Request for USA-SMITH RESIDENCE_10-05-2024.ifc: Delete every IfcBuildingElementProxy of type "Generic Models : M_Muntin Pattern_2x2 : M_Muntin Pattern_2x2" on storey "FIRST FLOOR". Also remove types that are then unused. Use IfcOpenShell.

First a look at what the model holds.

```python
import ifcopenshell
import ifcopenshell.util.element

model = ifcopenshell.open("USA-SMITH RESIDENCE_10-05-2024.ifc")
print(model.schema)
storey = next(s for s in model.by_type("IfcBuildingStorey") if s.Name == "FIRST FLOOR")
proxies = [e for e in ifcopenshell.util.element.get_decomposition(storey) if e.is_a("IfcBuildingElementProxy")]
seen = {}
for e in proxies:
    element_type = ifcopenshell.util.element.get_type(e)
    name = element_type.Name if element_type not in (None, e) else None
    seen[name] = seen.get(name, 0) + 1
for name, count in sorted(seen.items(), key=str):
    print(count, "x", name)
```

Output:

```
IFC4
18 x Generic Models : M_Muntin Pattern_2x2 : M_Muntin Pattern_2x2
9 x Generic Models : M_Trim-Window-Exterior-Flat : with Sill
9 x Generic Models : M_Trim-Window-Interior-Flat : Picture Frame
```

```python
import ifcopenshell
import ifcopenshell.api.root
import ifcopenshell.util.element

model = ifcopenshell.open("USA-SMITH RESIDENCE_10-05-2024.ifc")

storey = next(s for s in model.by_type("IfcBuildingStorey") if s.Name == "FIRST FLOOR")
proxies = [e for e in ifcopenshell.util.element.get_decomposition(storey) if e.is_a("IfcBuildingElementProxy")]
targets = [e for e in proxies if (t := ifcopenshell.util.element.get_type(e)) not in (None, e) and t.Name == "Generic Models : M_Muntin Pattern_2x2 : M_Muntin Pattern_2x2"]
types = {ifcopenshell.util.element.get_type(e) for e in targets} - {None, *targets}

for e in targets:
    ifcopenshell.api.root.remove_product(model, product=e)
print(len(targets), "removed")

unused = [t for t in types if not ifcopenshell.util.element.get_types(t)]
for t in unused:
    ifcopenshell.api.root.remove_product(model, product=t)
print(len(unused), "unused types removed")

model.write("USA-SMITH RESIDENCE_10-05-2024_edited.ifc")
```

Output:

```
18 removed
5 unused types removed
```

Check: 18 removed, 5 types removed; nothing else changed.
